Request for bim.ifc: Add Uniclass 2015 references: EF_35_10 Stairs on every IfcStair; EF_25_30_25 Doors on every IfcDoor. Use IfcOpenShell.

First a look at what the model holds.

```python
import ifcopenshell

model = ifcopenshell.open("bim.ifc")
print(model.schema)
print("classifications:", [c.Name for c in model.by_type("IfcClassification")])
for ifc_class in ("IfcDoor", "IfcRoof", "IfcStair", "IfcWall", "IfcWindow"):
    print(ifc_class, len(model.by_type(ifc_class)))
```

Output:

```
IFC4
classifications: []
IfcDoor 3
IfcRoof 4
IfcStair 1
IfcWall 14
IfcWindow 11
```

```python
import ifcopenshell
import ifcopenshell.api.classification

model = ifcopenshell.open("bim.ifc")

system = ifcopenshell.api.classification.add_classification(model, classification="Uniclass 2015")

codes = {
    "IfcStair": ("EF_35_10", "Stairs"),
    "IfcDoor": ("EF_25_30_25", "Doors"),
}
for ifc_class, (code, name) in codes.items():
    products = model.by_type(ifc_class)
    ifcopenshell.api.classification.add_reference(
        model, products=products, classification=system, identification=code, name=name
    )
    print(code, len(products))

model.write("bim_edited.ifc")
```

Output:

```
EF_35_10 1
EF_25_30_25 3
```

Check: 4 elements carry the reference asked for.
